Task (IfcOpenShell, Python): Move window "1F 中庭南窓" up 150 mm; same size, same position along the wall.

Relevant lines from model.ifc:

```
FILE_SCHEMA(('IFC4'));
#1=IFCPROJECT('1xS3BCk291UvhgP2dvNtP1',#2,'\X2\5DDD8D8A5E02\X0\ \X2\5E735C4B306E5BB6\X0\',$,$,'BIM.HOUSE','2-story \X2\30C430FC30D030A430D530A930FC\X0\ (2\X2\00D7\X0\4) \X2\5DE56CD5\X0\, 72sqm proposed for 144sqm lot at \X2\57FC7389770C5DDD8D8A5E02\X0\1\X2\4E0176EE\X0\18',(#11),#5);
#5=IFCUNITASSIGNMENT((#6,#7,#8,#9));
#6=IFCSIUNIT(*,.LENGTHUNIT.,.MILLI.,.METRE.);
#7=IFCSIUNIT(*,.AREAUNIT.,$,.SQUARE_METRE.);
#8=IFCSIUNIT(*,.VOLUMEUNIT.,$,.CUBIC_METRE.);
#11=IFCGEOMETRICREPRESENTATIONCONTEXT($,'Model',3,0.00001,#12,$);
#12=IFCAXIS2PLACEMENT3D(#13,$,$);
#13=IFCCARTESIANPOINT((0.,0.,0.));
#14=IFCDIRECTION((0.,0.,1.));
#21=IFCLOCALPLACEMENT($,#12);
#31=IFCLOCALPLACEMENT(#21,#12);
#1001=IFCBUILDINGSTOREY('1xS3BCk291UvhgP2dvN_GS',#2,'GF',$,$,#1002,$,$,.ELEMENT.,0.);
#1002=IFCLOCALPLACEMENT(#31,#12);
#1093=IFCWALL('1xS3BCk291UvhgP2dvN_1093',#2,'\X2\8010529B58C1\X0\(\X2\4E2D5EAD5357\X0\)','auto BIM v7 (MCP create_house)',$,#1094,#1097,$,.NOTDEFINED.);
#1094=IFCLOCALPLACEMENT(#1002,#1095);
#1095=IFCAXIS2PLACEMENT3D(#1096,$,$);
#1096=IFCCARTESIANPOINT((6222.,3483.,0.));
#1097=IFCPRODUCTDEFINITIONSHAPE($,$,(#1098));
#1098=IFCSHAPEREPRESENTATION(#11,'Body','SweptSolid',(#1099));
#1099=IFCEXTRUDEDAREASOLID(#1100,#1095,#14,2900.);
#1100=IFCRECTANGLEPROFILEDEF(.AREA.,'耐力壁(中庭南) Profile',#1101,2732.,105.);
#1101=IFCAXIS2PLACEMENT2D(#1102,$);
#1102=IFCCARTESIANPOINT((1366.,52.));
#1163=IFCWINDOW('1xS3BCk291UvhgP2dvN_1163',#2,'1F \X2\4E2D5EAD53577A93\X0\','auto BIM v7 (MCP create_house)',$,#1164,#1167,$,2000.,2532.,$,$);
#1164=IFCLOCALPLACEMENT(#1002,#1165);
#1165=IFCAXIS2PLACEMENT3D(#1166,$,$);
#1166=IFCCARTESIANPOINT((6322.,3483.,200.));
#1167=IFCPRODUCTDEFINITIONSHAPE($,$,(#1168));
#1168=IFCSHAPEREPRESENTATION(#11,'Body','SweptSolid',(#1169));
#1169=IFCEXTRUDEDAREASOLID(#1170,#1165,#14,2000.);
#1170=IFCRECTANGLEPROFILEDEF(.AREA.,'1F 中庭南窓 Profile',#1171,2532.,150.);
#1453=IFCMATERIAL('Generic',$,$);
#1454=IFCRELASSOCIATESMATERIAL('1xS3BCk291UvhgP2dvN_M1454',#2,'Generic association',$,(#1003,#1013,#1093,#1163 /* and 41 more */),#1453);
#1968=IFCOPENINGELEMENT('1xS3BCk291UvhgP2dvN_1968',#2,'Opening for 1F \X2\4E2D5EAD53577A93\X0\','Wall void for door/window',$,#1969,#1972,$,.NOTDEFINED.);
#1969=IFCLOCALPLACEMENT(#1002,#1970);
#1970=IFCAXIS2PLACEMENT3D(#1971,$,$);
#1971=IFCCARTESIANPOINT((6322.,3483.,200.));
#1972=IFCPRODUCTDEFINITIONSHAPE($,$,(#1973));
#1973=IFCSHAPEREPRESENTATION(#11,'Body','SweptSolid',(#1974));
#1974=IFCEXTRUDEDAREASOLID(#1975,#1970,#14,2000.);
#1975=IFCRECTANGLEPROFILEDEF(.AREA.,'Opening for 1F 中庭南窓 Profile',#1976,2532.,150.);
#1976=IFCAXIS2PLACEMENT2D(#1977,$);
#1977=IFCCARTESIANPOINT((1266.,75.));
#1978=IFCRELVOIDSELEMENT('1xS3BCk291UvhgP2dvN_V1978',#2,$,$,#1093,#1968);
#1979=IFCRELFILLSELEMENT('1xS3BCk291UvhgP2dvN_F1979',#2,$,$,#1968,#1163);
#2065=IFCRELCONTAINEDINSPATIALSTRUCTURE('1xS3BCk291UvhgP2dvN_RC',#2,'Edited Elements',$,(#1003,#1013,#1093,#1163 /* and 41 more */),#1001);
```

```python
import numpy as np
import ifcopenshell
import ifcopenshell.api.geometry
import ifcopenshell.util.placement
import ifcopenshell.util.unit

model = ifcopenshell.open("model.ifc")
unit_scale = ifcopenshell.util.unit.calculate_unit_scale(model)

window = model.by_id(1163)
opening = window.FillsVoids[0].RelatingOpeningElement
dz = 150.0

shift = np.array([0.0, 0.0, dz])
# The window is not placed relative to its opening, so move both.
for product in (opening, window):
    matrix = ifcopenshell.util.placement.get_local_placement(product.ObjectPlacement)
    matrix[:3, 3] += shift
    ifcopenshell.api.geometry.edit_object_placement(model, product=product, matrix=matrix, is_si=False)

print(f"moved by {dz * unit_scale:+.3f} m")

model.write("model_edited.ifc")
```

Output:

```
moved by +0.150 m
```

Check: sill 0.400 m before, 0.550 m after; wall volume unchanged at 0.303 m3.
